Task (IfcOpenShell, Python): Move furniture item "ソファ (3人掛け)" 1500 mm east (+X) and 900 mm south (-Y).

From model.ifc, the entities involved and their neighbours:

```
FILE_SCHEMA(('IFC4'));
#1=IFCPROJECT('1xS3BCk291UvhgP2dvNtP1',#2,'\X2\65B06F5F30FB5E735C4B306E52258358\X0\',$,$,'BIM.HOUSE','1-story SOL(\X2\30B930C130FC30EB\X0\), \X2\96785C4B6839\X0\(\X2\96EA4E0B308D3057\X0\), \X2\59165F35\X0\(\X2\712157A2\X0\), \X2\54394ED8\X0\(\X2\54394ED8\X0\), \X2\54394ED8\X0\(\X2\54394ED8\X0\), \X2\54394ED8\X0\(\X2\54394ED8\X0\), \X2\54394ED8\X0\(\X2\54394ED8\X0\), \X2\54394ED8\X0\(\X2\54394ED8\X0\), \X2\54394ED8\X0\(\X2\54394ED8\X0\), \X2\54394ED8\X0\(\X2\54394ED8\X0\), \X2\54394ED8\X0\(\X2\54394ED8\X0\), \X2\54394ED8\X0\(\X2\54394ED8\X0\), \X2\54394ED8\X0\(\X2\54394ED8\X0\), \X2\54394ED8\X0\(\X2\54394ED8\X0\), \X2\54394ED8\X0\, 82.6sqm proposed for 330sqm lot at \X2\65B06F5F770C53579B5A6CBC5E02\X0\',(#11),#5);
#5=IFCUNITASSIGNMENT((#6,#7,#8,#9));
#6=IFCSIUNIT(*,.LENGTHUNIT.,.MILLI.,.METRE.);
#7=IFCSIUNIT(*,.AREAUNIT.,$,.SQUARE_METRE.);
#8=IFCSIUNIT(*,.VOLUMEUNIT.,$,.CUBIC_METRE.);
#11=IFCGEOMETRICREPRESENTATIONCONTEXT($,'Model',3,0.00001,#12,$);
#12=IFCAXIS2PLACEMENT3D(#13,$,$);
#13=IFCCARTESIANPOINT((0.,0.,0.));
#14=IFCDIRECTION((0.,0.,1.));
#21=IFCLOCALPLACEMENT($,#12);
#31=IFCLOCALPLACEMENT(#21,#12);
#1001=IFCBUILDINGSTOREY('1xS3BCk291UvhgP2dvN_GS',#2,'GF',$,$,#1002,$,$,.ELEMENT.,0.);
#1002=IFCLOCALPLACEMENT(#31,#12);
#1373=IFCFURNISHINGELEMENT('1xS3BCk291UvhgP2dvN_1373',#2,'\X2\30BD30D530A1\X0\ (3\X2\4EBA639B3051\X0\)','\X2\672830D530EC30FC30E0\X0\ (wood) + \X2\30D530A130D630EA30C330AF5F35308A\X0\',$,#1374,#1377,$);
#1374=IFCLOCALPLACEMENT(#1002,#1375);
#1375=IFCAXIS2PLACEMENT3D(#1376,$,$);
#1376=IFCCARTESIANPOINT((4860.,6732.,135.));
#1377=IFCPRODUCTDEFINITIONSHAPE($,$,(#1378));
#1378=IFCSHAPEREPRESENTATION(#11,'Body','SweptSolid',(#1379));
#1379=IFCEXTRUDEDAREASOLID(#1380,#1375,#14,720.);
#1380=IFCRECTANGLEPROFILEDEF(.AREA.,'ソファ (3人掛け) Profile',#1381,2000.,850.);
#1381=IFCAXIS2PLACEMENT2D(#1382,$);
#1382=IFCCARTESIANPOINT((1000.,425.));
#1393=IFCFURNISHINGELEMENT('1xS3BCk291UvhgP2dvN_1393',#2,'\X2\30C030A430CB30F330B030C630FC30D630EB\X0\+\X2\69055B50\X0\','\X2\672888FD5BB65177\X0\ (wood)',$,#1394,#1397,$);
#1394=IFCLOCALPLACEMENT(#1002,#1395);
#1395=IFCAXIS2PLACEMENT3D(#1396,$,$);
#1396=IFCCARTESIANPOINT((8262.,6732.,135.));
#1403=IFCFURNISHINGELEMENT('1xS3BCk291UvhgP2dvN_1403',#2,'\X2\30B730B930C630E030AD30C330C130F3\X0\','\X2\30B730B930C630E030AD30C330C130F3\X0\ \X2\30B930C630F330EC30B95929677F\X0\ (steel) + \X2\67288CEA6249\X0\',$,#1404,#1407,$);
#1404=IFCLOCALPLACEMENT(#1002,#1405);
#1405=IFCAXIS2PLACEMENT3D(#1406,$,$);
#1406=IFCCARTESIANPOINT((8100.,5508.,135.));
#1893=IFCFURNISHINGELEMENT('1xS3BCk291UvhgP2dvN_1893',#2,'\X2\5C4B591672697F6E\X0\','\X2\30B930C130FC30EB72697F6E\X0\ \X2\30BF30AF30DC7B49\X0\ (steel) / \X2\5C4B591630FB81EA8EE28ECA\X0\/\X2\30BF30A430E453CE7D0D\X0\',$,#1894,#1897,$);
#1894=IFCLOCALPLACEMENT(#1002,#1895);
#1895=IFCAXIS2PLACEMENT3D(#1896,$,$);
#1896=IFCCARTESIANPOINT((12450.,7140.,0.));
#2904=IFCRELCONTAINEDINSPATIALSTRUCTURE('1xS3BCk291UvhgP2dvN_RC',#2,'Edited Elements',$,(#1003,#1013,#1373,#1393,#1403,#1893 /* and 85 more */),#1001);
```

```python
import ifcopenshell
import ifcopenshell.api.geometry
import ifcopenshell.util.placement
import ifcopenshell.util.unit

model = ifcopenshell.open("model.ifc")
unit_scale = ifcopenshell.util.unit.calculate_unit_scale(model)

item = model.by_guid("1xS3BCk291UvhgP2dvN_1373")
matrix = ifcopenshell.util.placement.get_local_placement(item.ObjectPlacement)
matrix[0, 3] += 1.5 / unit_scale
matrix[1, 3] -= 0.9 / unit_scale
ifcopenshell.api.geometry.edit_object_placement(model, product=item, matrix=matrix, is_si=False)

print(ifcopenshell.util.placement.get_local_placement(item.ObjectPlacement).round(3) + 0.0)

model.write("model_edited.ifc")
```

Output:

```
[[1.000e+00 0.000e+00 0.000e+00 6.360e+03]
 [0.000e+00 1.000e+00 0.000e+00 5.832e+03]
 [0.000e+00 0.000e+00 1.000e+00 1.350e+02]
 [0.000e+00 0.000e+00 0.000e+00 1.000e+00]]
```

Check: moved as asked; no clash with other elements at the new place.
